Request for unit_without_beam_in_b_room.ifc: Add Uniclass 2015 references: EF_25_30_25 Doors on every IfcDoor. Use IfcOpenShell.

First a look at what the model holds.

```python
import ifcopenshell

model = ifcopenshell.open("unit_without_beam_in_b_room.ifc")
print(model.schema)
print("classifications:", [c.Name for c in model.by_type("IfcClassification")])
for ifc_class in ("IfcDoor", "IfcRoof", "IfcStair", "IfcWall", "IfcWindow"):
    print(ifc_class, len(model.by_type(ifc_class)))
```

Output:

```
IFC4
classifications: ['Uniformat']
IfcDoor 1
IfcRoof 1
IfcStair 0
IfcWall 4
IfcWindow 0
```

```python
import ifcopenshell
import ifcopenshell.api.classification

model = ifcopenshell.open("unit_without_beam_in_b_room.ifc")

system = ifcopenshell.api.classification.add_classification(model, classification="Uniclass 2015")

codes = {
    "IfcDoor": ("EF_25_30_25", "Doors"),
}
for ifc_class, (code, name) in codes.items():
    products = model.by_type(ifc_class)
    ifcopenshell.api.classification.add_reference(
        model, products=products, classification=system, identification=code, name=name
    )
    print(code, len(products))

model.write("unit_without_beam_in_b_room_v2.ifc")
```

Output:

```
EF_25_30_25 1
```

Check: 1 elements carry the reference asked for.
